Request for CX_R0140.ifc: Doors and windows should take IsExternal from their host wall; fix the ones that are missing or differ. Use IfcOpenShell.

First a look at what the model holds.

```python
import ifcopenshell
import ifcopenshell.util.element

model = ifcopenshell.open("CX_R0140.ifc")
print(model.schema)
seen = {}
for e in model.by_type("IfcDoor") + model.by_type("IfcWindow"):
    if not e.FillsVoids:
        continue
    host = e.FillsVoids[0].RelatingOpeningElement.VoidsElements[0].RelatingBuildingElement
    own = ifcopenshell.util.element.get_pset(e, f"Pset_{e.is_a()[3:].removesuffix('StandardCase')}Common", "IsExternal")
    wall = ifcopenshell.util.element.get_pset(host, "Pset_WallCommon", "IsExternal")
    seen[e.is_a(), own, wall] = seen.get((e.is_a(), own, wall), 0) + 1
for (cls, own, wall), count in sorted(seen.items(), key=str):
    print(count, cls, "IsExternal:", own, "| host wall:", wall)
```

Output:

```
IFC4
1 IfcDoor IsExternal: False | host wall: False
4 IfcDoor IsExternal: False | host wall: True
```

```python
import ifcopenshell
import ifcopenshell.api.pset
import ifcopenshell.util.element

model = ifcopenshell.open("CX_R0140.ifc")

count = 0
for ifc_class, pset_name in (("IfcDoor", "Pset_DoorCommon"), ("IfcWindow", "Pset_WindowCommon")):
    for e in model.by_type(ifc_class):
        if not e.FillsVoids:
            continue
        host = e.FillsVoids[0].RelatingOpeningElement.VoidsElements[0].RelatingBuildingElement
        external = ifcopenshell.util.element.get_pset(host, "Pset_WallCommon", "IsExternal")
        if external is None or ifcopenshell.util.element.get_pset(e, pset_name, "IsExternal") == external:
            continue
        pset = ifcopenshell.api.pset.add_pset(model, product=e, name=pset_name)
        ifcopenshell.api.pset.edit_pset(model, pset=pset, properties={"IsExternal": external})
        count += 1

print(count, "updated")

model.write("CX_R0140-out.ifc")
```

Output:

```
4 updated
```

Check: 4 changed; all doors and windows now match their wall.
